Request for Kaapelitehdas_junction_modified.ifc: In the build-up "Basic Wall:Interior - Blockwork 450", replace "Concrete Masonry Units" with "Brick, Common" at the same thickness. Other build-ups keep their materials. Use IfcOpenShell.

First a look at what the model holds.

```python
import ifcopenshell
import ifcopenshell.util.element

model = ifcopenshell.open("Kaapelitehdas_junction_modified.ifc")
print(model.schema)
for layer_set in model.by_type("IfcMaterialLayerSet"):
    if layer_set.LayerSetName == "Basic Wall:Interior - Blockwork 450":
        for layer in layer_set.MaterialLayers:
            print(layer.id(), layer.Material and layer.Material.Name, layer.LayerThickness, sep=" | ")
        print(len(ifcopenshell.util.element.get_elements_by_material(model, layer_set)), "elements and types use it")
print(sorted(m.Name for m in model.by_type("IfcMaterial") if m.Name)[:60])
```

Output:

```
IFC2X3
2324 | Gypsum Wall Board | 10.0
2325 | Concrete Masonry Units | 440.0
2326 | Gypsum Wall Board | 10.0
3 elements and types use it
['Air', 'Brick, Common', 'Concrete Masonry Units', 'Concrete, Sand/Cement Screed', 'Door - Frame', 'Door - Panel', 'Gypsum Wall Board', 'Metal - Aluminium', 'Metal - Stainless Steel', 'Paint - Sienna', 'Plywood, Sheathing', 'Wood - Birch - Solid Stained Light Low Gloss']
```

```python
import ifcopenshell
import ifcopenshell.api.material

model = ifcopenshell.open("Kaapelitehdas_junction_modified.ifc")

layer_set = next(s for s in model.by_type("IfcMaterialLayerSet") if s.LayerSetName == "Basic Wall:Interior - Blockwork 450")
layer = next(l for l in layer_set.MaterialLayers if l.Material and l.Material.Name == "Concrete Masonry Units")
material = next(m for m in model.by_type("IfcMaterial") if m.Name == "Brick, Common")

# Point this one layer at the other material; renaming the old one would change it everywhere.
ifcopenshell.api.material.edit_layer(model, layer=layer, attributes={}, material=material)

print([l.Material.Name if l.Material else None for l in layer_set.MaterialLayers])

model.write("Kaapelitehdas_junction_modified-out.ifc")
```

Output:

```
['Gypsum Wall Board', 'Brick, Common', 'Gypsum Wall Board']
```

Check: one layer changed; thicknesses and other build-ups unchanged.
